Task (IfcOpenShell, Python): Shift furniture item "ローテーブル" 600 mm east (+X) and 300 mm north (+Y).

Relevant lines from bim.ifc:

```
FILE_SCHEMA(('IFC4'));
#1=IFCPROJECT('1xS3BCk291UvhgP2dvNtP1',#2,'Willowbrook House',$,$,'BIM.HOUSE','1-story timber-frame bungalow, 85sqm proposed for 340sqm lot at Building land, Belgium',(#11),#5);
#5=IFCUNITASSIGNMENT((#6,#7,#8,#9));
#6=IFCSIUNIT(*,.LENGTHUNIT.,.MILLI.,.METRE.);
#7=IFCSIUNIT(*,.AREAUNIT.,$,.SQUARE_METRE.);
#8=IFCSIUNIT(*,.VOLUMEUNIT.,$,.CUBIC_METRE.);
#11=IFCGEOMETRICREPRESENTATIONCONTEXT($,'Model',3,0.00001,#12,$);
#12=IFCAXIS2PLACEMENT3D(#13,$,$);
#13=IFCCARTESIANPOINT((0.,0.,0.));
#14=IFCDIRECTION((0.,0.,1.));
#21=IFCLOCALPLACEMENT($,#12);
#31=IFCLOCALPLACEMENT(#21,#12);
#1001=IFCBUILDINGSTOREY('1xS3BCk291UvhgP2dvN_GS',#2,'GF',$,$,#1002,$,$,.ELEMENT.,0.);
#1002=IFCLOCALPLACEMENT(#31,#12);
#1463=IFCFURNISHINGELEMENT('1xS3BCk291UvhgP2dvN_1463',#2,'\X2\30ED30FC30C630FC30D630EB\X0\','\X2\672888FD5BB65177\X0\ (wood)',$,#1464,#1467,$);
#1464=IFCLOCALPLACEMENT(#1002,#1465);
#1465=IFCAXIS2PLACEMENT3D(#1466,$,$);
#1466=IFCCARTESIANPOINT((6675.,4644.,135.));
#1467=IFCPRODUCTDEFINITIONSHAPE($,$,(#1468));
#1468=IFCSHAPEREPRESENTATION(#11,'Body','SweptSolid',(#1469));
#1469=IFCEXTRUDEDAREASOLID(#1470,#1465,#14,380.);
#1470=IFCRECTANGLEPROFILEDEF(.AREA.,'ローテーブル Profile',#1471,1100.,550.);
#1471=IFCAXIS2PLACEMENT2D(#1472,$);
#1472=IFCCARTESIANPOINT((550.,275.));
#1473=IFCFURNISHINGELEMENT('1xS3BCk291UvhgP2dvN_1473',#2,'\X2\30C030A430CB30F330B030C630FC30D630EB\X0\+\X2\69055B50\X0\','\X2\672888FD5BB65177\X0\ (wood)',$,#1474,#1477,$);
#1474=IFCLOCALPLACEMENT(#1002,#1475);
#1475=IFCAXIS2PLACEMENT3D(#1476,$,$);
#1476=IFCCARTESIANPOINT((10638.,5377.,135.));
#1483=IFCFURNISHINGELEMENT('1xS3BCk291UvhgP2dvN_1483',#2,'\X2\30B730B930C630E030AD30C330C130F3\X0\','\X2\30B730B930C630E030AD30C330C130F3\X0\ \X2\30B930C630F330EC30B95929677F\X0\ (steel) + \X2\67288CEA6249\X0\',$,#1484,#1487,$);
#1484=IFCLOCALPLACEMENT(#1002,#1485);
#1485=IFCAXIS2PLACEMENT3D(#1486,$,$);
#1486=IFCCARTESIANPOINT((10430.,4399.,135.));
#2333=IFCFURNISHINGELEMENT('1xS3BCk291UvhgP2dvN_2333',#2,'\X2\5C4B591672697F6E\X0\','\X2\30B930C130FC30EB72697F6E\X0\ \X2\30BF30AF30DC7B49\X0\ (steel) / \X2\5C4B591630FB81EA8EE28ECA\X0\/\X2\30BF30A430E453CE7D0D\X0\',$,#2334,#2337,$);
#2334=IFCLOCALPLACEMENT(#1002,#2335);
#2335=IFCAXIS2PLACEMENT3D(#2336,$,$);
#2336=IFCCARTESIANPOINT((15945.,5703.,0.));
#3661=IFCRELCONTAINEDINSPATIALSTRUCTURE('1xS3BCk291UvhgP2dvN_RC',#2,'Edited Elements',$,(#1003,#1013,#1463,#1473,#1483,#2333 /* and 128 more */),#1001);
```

```python
import ifcopenshell
import ifcopenshell.api.geometry
import ifcopenshell.util.placement
import ifcopenshell.util.unit

model = ifcopenshell.open("bim.ifc")
unit_scale = ifcopenshell.util.unit.calculate_unit_scale(model)

item = model.by_guid("1xS3BCk291UvhgP2dvN_1463")
matrix = ifcopenshell.util.placement.get_local_placement(item.ObjectPlacement)
matrix[0, 3] += 0.6 / unit_scale
matrix[1, 3] += 0.3 / unit_scale
ifcopenshell.api.geometry.edit_object_placement(model, product=item, matrix=matrix, is_si=False)

print(ifcopenshell.util.placement.get_local_placement(item.ObjectPlacement).round(3) + 0.0)

model.write("bim_rev.ifc")
```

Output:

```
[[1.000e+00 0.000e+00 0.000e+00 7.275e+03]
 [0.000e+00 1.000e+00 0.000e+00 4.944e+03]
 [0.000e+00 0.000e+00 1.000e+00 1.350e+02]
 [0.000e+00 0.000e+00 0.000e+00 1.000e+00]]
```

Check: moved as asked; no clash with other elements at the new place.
